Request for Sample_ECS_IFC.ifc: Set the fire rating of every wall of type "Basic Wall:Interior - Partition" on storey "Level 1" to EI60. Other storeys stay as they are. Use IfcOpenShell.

First a look at what the model holds.

```python
import ifcopenshell
import ifcopenshell.util.element

model = ifcopenshell.open("Sample_ECS_IFC.ifc")
print(model.schema)
storey = next(s for s in model.by_type("IfcBuildingStorey") if s.Name == "Level 1")
walls = [e for e in ifcopenshell.util.element.get_decomposition(storey) if e.is_a("IfcWall")]
seen = {}
for e in walls:
    element_type = ifcopenshell.util.element.get_type(e)
    key = (element_type.Name if element_type != e and element_type else None, ifcopenshell.util.element.get_pset(e, "Pset_WallCommon", "FireRating"))
    seen[key] = seen.get(key, 0) + 1
for (name, value), count in sorted(seen.items(), key=str):
    print(count, "x", name, "|", value)
```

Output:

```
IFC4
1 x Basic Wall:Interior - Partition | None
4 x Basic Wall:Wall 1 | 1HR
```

```python
import ifcopenshell
import ifcopenshell.api.pset
import ifcopenshell.util.element

model = ifcopenshell.open("Sample_ECS_IFC.ifc")

storey = next(s for s in model.by_type("IfcBuildingStorey") if s.Name == "Level 1")
walls = [e for e in ifcopenshell.util.element.get_decomposition(storey) if e.is_a("IfcWall")]

count = 0
for e in walls:
    element_type = ifcopenshell.util.element.get_type(e)
    if element_type in (None, e) or element_type.Name != "Basic Wall:Interior - Partition":
        continue
    # add_pset returns the element's existing set when there is one.
    pset = ifcopenshell.api.pset.add_pset(model, product=e, name="Pset_WallCommon")
    ifcopenshell.api.pset.edit_pset(model, pset=pset, properties={"FireRating": "EI60"})
    count += 1

print(count, "walls updated")

model.write("Sample_ECS_IFC_updated.ifc")
```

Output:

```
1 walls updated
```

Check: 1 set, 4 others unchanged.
